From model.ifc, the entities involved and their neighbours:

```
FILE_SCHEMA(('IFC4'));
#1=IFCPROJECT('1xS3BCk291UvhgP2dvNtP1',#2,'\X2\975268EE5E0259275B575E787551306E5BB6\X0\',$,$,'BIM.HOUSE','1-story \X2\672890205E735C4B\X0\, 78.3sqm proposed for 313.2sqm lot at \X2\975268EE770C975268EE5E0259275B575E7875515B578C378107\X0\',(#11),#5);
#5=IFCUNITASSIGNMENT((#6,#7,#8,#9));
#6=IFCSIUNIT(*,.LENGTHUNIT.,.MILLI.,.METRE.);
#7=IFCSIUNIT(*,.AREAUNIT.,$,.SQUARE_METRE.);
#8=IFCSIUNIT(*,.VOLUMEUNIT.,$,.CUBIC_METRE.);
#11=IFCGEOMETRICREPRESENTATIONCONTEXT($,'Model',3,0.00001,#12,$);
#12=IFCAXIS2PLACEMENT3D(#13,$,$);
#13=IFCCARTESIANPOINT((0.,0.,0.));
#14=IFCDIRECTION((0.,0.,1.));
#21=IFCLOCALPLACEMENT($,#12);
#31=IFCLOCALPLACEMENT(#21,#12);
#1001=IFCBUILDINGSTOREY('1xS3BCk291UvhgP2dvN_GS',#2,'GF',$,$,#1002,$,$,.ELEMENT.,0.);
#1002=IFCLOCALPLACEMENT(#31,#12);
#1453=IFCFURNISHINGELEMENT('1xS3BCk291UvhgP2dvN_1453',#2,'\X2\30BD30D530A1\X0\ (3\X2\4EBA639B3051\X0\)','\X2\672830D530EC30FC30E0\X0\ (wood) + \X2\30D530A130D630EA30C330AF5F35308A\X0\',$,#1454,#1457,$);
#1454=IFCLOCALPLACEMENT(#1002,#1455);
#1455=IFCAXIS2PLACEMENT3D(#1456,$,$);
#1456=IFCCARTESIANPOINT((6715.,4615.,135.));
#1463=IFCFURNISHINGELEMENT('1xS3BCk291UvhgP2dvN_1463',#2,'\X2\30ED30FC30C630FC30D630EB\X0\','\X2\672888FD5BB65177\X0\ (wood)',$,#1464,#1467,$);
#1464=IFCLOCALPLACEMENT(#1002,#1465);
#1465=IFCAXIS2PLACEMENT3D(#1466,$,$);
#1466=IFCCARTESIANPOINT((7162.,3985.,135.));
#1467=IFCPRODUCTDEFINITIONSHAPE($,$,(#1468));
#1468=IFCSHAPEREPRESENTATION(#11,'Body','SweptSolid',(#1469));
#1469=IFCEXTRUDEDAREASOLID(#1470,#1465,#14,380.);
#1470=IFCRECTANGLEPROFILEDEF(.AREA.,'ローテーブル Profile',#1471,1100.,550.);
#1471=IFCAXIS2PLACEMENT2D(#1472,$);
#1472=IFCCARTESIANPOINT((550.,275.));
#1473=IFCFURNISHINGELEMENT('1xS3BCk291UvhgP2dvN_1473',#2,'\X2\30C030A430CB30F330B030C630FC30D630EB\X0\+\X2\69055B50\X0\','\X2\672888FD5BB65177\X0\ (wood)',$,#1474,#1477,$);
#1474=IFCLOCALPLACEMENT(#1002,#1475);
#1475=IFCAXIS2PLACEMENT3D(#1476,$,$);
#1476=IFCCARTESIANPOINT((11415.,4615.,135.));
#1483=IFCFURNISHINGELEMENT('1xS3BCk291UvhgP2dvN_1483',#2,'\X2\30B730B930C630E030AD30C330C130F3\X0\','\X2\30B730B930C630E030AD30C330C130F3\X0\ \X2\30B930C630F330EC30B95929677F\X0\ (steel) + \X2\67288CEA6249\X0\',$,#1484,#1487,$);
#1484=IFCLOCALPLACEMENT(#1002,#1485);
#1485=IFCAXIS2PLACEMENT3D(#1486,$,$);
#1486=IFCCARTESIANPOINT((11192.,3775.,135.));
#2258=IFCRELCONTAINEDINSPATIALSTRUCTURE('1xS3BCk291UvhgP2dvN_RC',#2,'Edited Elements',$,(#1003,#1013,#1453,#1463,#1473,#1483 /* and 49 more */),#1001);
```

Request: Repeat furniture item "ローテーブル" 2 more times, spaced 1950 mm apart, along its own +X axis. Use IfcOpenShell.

```python
import ifcopenshell
import ifcopenshell.api.geometry
import ifcopenshell.api.root
import ifcopenshell.util.element
import ifcopenshell.util.placement
import ifcopenshell.util.unit

model = ifcopenshell.open("model.ifc")
unit_scale = ifcopenshell.util.unit.calculate_unit_scale(model)


def reuse_history(source, copy):
    """copy_class also copies each property set's owner history, people and application; keep the originals."""
    for rel in copy.IsDefinedBy:
        if rel.is_a("IfcRelDefinesByProperties") and (history := rel.RelatingPropertyDefinition.OwnerHistory):
            rel.RelatingPropertyDefinition.OwnerHistory = source.OwnerHistory
            ifcopenshell.util.element.remove_deep2(model, history)


source = model.by_guid("1xS3BCk291UvhgP2dvN_1463")
base = ifcopenshell.util.placement.get_local_placement(source.ObjectPlacement)
step = base[:3, 0] * 1.95 / unit_scale

for i in range(1, 3):
    copy = ifcopenshell.api.root.copy_class(model, product=source)
    copy.Representation = ifcopenshell.util.element.copy_deep(
        model, source.Representation, exclude=["IfcGeometricRepresentationContext", "IfcRepresentationMap"]
    )
    reuse_history(source, copy)
    matrix = base.copy()
    matrix[:3, 3] += i * step
    print("added at", matrix[:3, 3].round(3) + 0.0)
    ifcopenshell.api.geometry.edit_object_placement(model, product=copy, matrix=matrix, is_si=False)

model.write("model_updated.ifc")
```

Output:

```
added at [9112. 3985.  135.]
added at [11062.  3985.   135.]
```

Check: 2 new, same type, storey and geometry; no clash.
